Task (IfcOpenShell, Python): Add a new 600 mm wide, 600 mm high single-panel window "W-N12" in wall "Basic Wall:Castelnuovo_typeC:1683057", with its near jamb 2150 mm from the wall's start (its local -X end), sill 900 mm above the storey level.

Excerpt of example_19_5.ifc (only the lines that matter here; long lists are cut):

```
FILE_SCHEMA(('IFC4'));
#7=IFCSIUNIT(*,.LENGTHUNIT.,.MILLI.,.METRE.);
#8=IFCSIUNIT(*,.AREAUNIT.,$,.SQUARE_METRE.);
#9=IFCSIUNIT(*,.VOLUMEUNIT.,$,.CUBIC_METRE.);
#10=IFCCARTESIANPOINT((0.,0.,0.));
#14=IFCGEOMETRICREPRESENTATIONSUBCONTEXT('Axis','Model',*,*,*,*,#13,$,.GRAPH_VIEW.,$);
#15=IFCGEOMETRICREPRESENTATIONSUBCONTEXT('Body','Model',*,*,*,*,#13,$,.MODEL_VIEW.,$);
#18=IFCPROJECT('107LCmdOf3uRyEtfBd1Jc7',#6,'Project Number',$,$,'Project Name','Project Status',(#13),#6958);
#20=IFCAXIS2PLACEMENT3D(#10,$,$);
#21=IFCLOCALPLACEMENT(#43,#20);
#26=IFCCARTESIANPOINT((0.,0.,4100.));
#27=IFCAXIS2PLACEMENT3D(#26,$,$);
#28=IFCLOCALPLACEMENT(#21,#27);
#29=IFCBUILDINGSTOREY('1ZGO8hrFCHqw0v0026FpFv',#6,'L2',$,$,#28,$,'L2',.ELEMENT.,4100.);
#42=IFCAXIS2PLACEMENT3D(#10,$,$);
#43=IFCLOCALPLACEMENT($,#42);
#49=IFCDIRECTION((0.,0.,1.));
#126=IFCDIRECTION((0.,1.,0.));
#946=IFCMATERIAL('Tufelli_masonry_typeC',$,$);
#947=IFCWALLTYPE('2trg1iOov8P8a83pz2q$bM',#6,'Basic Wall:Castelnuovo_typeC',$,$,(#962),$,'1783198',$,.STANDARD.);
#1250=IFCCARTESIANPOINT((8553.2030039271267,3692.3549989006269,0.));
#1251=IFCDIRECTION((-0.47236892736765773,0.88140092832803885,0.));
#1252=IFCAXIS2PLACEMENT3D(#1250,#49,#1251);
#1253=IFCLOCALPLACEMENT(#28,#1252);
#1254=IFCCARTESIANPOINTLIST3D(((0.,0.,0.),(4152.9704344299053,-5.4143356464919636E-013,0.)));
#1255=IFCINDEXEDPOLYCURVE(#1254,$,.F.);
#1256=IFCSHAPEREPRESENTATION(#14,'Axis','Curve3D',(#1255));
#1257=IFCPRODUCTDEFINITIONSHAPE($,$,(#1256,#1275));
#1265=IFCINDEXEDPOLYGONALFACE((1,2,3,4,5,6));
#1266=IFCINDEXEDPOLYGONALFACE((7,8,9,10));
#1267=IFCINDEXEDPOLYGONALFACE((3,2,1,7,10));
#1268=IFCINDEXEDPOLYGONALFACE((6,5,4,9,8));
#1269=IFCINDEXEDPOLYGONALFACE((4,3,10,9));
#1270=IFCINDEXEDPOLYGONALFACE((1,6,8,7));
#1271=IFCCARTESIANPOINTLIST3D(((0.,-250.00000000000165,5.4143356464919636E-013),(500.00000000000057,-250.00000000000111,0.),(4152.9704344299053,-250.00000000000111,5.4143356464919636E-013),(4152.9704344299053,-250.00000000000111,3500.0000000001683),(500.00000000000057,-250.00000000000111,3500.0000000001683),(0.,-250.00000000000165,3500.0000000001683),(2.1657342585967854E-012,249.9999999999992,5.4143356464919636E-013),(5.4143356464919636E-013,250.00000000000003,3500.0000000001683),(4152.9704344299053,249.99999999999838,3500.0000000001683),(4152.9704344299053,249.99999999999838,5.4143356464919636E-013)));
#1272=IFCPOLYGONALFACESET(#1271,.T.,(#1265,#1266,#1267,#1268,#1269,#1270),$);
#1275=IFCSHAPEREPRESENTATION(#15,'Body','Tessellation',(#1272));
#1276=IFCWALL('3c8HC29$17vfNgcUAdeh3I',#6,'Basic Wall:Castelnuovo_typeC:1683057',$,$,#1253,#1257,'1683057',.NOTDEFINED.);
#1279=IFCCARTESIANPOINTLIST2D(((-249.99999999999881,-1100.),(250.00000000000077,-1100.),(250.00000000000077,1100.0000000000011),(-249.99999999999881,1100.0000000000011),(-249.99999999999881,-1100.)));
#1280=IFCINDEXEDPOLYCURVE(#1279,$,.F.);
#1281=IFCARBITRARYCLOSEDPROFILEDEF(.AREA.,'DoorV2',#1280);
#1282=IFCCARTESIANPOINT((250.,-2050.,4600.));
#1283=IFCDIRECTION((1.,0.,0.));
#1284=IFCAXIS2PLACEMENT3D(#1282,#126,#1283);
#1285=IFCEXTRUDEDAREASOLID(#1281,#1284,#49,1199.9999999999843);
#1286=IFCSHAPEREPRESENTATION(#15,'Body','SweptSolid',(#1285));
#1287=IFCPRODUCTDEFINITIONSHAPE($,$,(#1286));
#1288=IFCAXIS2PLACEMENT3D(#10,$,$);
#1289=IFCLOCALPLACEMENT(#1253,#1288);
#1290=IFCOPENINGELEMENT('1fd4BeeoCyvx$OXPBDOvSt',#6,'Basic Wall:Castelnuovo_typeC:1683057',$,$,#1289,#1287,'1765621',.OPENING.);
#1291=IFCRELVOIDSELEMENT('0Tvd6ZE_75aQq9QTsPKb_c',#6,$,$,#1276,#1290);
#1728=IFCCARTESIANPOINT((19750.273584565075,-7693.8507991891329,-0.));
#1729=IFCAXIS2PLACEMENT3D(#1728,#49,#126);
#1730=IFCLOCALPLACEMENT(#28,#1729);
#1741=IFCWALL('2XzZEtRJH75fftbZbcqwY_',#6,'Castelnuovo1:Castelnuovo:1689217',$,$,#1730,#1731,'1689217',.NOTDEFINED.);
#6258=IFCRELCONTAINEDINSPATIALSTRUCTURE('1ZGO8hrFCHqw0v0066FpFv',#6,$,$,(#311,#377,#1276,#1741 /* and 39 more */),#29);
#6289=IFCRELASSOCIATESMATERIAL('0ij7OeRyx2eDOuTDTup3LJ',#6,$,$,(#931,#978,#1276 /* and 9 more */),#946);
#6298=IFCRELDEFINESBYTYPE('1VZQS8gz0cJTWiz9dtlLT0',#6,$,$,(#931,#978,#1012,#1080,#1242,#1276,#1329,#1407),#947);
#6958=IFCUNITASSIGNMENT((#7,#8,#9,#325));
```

```python
import numpy as np
import ifcopenshell
import ifcopenshell.api.feature
import ifcopenshell.api.geometry
import ifcopenshell.api.root
import ifcopenshell.api.spatial
import ifcopenshell.geom
import ifcopenshell.util.element
import ifcopenshell.util.placement
import ifcopenshell.util.representation
import ifcopenshell.util.shape
import ifcopenshell.util.unit

model = ifcopenshell.open("example_19_5.ifc")
unit_scale = ifcopenshell.util.unit.calculate_unit_scale(model)
settings = ifcopenshell.geom.settings()


def volume(element):
    """Net volume in cubic metres, openings subtracted."""
    shape = ifcopenshell.geom.create_shape(settings, element)
    return ifcopenshell.util.shape.get_volume(shape.geometry)


wall = model.by_guid("3c8HC29$17vfNgcUAdeh3I")
storey = ifcopenshell.util.element.get_container(wall, ifc_class="IfcBuildingStorey")
context = ifcopenshell.util.representation.get_context(model, "Model", "Body", "MODEL_VIEW")
before = volume(wall)

width, height, from_end, sill = 0.6, 0.6, 2.15, 0.9  # metres

# The wall runs along its own X axis, and the end named is its -X end.
wall_shape = ifcopenshell.geom.create_shape(settings, wall)
x, y, z = ifcopenshell.util.shape.get_vertices(wall_shape.geometry).T
start = x.min() + from_end
face, thickness = float(y.min()), float(y.max() - y.min())
wall_matrix = ifcopenshell.util.placement.get_local_placement(wall.ObjectPlacement)
level = ifcopenshell.util.placement.get_local_placement(storey.ObjectPlacement)[2, 3]


def in_wall(x, y):
    """Placement at x, y metres in the wall's axes, at sill height."""
    matrix = wall_matrix.copy()
    matrix[:, 3] = wall_matrix @ np.array([x / unit_scale, y / unit_scale, 0.0, 1.0])
    matrix[2, 3] = level + sill / unit_scale
    return matrix


# Opening: a box that overshoots both wall faces by 50 mm.
opening = ifcopenshell.api.root.create_entity(model, ifc_class="IfcOpeningElement", predefined_type="OPENING")
box = ifcopenshell.api.geometry.add_wall_representation(
    model, context=context, length=width, height=height, thickness=thickness + 0.1
)
ifcopenshell.api.geometry.assign_representation(model, product=opening, representation=box)
ifcopenshell.api.geometry.edit_object_placement(model, product=opening, matrix=in_wall(start, face - 0.05), is_si=False)
ifcopenshell.api.feature.add_feature(model, feature=opening, element=wall)

window = ifcopenshell.api.root.create_entity(model, ifc_class="IfcWindow", name="W-N12", predefined_type="WINDOW")
window.OverallWidth, window.OverallHeight = width / unit_scale, height / unit_scale
window.PartitioningType = "SINGLE_PANEL"
body = ifcopenshell.api.geometry.add_window_representation(
    model,
    context=context,
    overall_width=window.OverallWidth,
    overall_height=window.OverallHeight,
    partition_type="SINGLE_PANEL",
)
ifcopenshell.api.geometry.assign_representation(model, product=window, representation=body)
ifcopenshell.api.spatial.assign_container(model, products=[window], relating_structure=storey)
ifcopenshell.api.feature.add_filling(model, opening=opening, element=window)

# Centre the window in the wall's thickness.
ifcopenshell.api.geometry.edit_object_placement(model, product=window, matrix=in_wall(start, face), is_si=False)
window_shape = ifcopenshell.geom.create_shape(settings, window)
depth = ifcopenshell.util.shape.get_vertices(window_shape.geometry)[:, 1]
offset = face + thickness / 2 - (depth.min() + depth.max()) / 2
ifcopenshell.api.geometry.edit_object_placement(model, product=window, matrix=in_wall(start, offset), is_si=False)

after = volume(wall)

print(f"wall volume {before:.3f} -> {after:.3f} m3")

model.write("example_19_5_rev.ifc")
```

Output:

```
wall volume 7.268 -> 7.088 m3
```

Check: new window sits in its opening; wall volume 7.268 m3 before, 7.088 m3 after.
